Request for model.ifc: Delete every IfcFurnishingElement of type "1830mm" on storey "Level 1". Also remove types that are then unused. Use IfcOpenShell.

First a look at what the model holds.

```python
import ifcopenshell
import ifcopenshell.util.element

model = ifcopenshell.open("model.ifc")
print(model.schema)
storey = next(s for s in model.by_type("IfcBuildingStorey") if s.Name == "Level 1")
furniture = [e for e in ifcopenshell.util.element.get_decomposition(storey) if e.is_a("IfcFurnishingElement")]
seen = {}
for e in furniture:
    element_type = ifcopenshell.util.element.get_type(e)
    name = element_type.Name if element_type not in (None, e) else None
    seen[name] = seen.get(name, 0) + 1
for name, count in sorted(seen.items(), key=str):
    print(count, "x", name)
```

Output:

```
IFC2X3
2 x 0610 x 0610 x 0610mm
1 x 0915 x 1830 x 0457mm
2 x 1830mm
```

```python
import ifcopenshell
import ifcopenshell.api.root
import ifcopenshell.util.element

model = ifcopenshell.open("model.ifc")

storey = next(s for s in model.by_type("IfcBuildingStorey") if s.Name == "Level 1")
furniture = [e for e in ifcopenshell.util.element.get_decomposition(storey) if e.is_a("IfcFurnishingElement")]
targets = [e for e in furniture if (t := ifcopenshell.util.element.get_type(e)) not in (None, e) and t.Name == "1830mm"]
types = {ifcopenshell.util.element.get_type(e) for e in targets} - {None, *targets}

for e in targets:
    ifcopenshell.api.root.remove_product(model, product=e)
print(len(targets), "removed")

unused = [t for t in types if not ifcopenshell.util.element.get_types(t)]
for t in unused:
    ifcopenshell.api.root.remove_product(model, product=t)
print(len(unused), "unused types removed")

model.write("model-out.ifc")
```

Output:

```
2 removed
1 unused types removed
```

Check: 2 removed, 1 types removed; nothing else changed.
